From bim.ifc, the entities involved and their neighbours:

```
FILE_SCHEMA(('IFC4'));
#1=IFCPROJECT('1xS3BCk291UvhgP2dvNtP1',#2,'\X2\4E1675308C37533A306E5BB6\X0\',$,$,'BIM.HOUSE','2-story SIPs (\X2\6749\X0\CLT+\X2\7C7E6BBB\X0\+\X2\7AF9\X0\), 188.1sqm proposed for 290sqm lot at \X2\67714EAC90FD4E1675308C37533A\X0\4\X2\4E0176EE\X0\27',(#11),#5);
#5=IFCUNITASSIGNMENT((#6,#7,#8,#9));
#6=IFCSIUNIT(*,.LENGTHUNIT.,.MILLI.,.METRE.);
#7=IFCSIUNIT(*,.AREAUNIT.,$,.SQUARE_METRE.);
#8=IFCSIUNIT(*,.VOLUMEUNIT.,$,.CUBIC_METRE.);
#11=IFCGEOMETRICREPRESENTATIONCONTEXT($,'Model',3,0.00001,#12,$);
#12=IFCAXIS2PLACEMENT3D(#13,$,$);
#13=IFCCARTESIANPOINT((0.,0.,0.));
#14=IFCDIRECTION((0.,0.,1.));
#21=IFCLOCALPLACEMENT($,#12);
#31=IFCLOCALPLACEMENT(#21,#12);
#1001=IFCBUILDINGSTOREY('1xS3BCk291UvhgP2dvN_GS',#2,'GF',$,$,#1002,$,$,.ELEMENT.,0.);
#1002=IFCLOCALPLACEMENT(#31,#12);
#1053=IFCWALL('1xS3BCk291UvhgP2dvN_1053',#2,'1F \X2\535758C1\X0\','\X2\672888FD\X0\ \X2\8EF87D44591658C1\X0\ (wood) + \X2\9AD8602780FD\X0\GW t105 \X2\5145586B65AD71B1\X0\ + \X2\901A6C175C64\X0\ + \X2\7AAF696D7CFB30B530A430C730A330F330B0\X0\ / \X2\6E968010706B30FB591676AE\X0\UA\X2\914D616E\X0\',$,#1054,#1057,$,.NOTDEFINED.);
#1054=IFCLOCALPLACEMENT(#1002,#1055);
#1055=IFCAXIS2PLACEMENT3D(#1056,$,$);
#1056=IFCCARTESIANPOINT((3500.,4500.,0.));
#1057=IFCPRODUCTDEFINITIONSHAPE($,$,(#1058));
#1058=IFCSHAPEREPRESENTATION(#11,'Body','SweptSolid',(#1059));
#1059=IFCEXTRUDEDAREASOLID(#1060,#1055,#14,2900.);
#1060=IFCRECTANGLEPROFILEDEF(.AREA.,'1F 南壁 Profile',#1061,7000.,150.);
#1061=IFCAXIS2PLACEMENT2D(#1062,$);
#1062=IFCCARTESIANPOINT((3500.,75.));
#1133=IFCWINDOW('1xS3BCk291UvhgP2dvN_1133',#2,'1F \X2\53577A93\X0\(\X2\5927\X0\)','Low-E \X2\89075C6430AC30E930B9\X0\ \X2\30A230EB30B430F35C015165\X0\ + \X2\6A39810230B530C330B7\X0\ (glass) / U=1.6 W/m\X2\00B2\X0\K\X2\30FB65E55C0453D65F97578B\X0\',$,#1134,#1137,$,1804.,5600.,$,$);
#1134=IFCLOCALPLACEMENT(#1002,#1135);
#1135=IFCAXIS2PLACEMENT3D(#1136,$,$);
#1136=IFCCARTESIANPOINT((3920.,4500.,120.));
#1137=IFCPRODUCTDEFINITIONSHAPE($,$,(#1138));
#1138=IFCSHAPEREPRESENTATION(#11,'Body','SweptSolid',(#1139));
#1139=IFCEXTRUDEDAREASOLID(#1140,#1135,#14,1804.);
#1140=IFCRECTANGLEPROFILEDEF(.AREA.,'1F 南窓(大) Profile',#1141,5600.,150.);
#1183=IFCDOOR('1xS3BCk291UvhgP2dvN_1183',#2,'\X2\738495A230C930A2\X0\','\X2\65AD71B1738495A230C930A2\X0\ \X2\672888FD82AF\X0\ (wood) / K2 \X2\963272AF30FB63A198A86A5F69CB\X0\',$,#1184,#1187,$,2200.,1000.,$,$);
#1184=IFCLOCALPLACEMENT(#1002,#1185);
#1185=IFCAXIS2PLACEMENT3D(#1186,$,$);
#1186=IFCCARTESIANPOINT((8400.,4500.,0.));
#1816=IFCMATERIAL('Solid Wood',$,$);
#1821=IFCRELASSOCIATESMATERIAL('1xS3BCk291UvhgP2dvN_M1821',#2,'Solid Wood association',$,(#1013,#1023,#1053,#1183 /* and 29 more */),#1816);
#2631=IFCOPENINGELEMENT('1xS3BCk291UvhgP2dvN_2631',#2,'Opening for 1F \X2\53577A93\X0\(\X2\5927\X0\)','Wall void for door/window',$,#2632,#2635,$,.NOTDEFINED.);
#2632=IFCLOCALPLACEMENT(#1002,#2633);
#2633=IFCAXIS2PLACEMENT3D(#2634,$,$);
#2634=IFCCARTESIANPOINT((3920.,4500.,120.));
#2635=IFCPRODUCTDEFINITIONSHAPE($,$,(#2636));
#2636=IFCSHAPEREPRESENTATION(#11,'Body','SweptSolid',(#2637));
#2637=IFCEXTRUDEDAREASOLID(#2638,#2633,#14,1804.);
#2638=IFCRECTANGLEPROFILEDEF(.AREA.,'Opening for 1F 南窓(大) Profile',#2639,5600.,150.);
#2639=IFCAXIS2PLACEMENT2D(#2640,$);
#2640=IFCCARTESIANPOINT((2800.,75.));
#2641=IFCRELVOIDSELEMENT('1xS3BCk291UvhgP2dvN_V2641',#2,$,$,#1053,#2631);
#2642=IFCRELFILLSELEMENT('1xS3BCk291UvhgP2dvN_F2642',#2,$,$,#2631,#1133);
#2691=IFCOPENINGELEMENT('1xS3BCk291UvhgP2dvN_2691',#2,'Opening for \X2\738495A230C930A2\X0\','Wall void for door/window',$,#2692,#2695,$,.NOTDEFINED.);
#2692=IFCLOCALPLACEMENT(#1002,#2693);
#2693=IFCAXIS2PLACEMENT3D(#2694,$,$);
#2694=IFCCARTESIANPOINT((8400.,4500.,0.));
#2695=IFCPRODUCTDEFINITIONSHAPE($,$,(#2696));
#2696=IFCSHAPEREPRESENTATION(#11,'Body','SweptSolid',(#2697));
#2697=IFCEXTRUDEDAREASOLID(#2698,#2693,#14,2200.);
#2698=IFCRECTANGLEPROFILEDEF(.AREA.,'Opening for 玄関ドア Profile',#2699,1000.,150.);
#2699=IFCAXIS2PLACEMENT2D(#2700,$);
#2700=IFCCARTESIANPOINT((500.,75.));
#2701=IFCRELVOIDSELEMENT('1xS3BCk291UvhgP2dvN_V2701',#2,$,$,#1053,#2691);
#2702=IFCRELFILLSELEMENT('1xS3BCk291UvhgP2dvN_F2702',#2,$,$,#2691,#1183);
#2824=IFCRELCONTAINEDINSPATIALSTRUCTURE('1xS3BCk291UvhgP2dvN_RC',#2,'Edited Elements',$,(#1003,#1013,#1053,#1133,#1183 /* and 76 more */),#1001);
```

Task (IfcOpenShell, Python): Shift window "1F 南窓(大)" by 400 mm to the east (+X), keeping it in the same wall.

```python
import ifcopenshell
import ifcopenshell.api.geometry
import ifcopenshell.util.placement
import ifcopenshell.util.unit

model = ifcopenshell.open("bim.ifc")
unit_scale = ifcopenshell.util.unit.calculate_unit_scale(model)

window = model.by_guid("1xS3BCk291UvhgP2dvN_1133")
opening = window.FillsVoids[0].RelatingOpeningElement
wall = opening.VoidsElements[0].RelatingBuildingElement

wall_matrix = ifcopenshell.util.placement.get_local_placement(wall.ObjectPlacement)
shift = wall_matrix[:3, 0] * 0.4 / unit_scale
before = ifcopenshell.util.placement.get_local_placement(window.ObjectPlacement)[:3, 3].copy()

# The window is not placed relative to its opening, so move both.
for product in (opening, window):
    matrix = ifcopenshell.util.placement.get_local_placement(product.ObjectPlacement)
    matrix[:3, 3] += shift
    ifcopenshell.api.geometry.edit_object_placement(model, product=product, matrix=matrix, is_si=False)

after = ifcopenshell.util.placement.get_local_placement(window.ObjectPlacement)[:3, 3]
print("window moved by", (after - before).round(3) + 0.0)

model.write("bim_edited.ifc")
```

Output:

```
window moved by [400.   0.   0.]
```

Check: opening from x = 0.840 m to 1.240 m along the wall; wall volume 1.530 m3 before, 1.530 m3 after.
